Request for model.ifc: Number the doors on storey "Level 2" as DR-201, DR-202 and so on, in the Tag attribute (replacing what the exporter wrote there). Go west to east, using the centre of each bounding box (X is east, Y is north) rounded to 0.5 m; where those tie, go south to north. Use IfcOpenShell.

First a look at what the model holds.

```python
import ifcopenshell
import ifcopenshell.util.element
import ifcopenshell.util.placement

model = ifcopenshell.open("model.ifc")
print(model.schema)
storey = next(s for s in model.by_type("IfcBuildingStorey") if s.Name == "Level 2")
doors = [e for e in ifcopenshell.util.element.get_decomposition(storey) if e.is_a("IfcDoor")]
for e in sorted(doors, key=lambda e: e.id()):
    origin = ifcopenshell.util.placement.get_local_placement(e.ObjectPlacement)[:3, 3]
    print(e.id(), e.Tag, e.Name, origin.round(2) + 0.0, sep=" | ")
```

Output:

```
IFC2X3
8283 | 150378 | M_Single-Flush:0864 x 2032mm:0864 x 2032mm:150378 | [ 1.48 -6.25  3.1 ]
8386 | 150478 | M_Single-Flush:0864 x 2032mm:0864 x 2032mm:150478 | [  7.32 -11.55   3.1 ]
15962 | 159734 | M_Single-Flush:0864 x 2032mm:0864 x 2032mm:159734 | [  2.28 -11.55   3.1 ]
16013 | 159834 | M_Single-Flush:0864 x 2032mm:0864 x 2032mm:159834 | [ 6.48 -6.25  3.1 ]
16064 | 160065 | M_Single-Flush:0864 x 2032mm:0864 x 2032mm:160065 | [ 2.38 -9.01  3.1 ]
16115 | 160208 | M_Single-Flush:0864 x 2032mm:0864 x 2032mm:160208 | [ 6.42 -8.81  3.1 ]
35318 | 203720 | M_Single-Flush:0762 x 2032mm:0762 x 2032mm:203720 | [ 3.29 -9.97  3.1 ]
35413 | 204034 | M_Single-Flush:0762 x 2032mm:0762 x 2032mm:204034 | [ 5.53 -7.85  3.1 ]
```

```python
import ifcopenshell
import ifcopenshell.geom
import ifcopenshell.util.element
import ifcopenshell.util.shape

model = ifcopenshell.open("model.ifc")
settings = ifcopenshell.geom.settings()
settings.set("use-world-coords", True)


def centre(element):
    shape = ifcopenshell.geom.create_shape(settings, element)
    return ifcopenshell.util.shape.get_bbox_centroid(shape.geometry)


storey = next(s for s in model.by_type("IfcBuildingStorey") if s.Name == "Level 2")
doors = [e for e in ifcopenshell.util.element.get_decomposition(storey) if e.is_a("IfcDoor")]

# Insertion points can sit at a corner or the storey origin, so sort by the geometry (in metres).
centres = {e: centre(e) for e in doors}
doors.sort(key=lambda e: (round(centres[e][0] / 0.5), centres[e][1]))

for i, e in enumerate(doors, start=1):
    number = f"DR-2{i:02d}"
    e.Tag = number
    print(e.id(), number)

model.write("model-out.ifc")
```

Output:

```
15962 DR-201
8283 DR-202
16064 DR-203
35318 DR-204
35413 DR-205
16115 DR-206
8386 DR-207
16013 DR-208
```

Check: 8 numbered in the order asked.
